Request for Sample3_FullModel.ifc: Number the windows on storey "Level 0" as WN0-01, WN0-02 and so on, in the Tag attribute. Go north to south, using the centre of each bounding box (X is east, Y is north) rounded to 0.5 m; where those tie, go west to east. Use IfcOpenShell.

First a look at what the model holds.

```python
import ifcopenshell
import ifcopenshell.util.element
import ifcopenshell.util.placement

model = ifcopenshell.open("Sample3_FullModel.ifc")
print(model.schema)
storey = next(s for s in model.by_type("IfcBuildingStorey") if s.Name == "Level 0")
windows = [e for e in ifcopenshell.util.element.get_decomposition(storey) if e.is_a("IfcWindow")]
for e in sorted(windows, key=lambda e: e.id()):
    origin = ifcopenshell.util.placement.get_local_placement(e.ObjectPlacement)[:3, 3]
    print(e.id(), e.Tag, e.Name, origin.round(2) + 0.0, sep=" | ")
```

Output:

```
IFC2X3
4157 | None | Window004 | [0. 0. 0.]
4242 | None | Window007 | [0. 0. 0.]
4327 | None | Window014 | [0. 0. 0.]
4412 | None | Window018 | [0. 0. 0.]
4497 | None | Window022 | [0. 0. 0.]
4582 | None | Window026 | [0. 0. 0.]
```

```python
import ifcopenshell
import ifcopenshell.geom
import ifcopenshell.util.element
import ifcopenshell.util.shape

model = ifcopenshell.open("Sample3_FullModel.ifc")
settings = ifcopenshell.geom.settings()
settings.set("use-world-coords", True)


def centre(element):
    shape = ifcopenshell.geom.create_shape(settings, element)
    return ifcopenshell.util.shape.get_bbox_centroid(shape.geometry)


storey = next(s for s in model.by_type("IfcBuildingStorey") if s.Name == "Level 0")
windows = [e for e in ifcopenshell.util.element.get_decomposition(storey) if e.is_a("IfcWindow")]

# Insertion points can sit at a corner or the storey origin, so sort by the geometry (in metres).
centres = {e: centre(e) for e in windows}
windows.sort(key=lambda e: (-round(centres[e][1] / 0.5), centres[e][0]))

for i, e in enumerate(windows, start=1):
    number = f"WN0-{i:02d}"
    e.Tag = number
    print(e.id(), number)

model.write("Sample3_FullModel-out.ifc")
```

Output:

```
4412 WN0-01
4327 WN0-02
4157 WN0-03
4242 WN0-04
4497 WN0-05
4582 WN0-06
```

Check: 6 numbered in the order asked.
